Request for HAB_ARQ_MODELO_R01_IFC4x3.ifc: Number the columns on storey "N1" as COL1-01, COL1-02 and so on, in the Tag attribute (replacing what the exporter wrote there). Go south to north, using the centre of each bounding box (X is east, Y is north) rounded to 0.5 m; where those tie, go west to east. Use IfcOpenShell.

First a look at what the model holds.

```python
import ifcopenshell
import ifcopenshell.util.element
import ifcopenshell.util.placement

model = ifcopenshell.open("HAB_ARQ_MODELO_R01_IFC4x3.ifc")
print(model.schema)
storey = next(s for s in model.by_type("IfcBuildingStorey") if s.Name == "N1")
columns = [e for e in ifcopenshell.util.element.get_decomposition(storey) if e.is_a("IfcColumn")]
for e in sorted(columns, key=lambda e: e.id()):
    origin = ifcopenshell.util.placement.get_local_placement(e.ObjectPlacement)[:3, 3]
    print(e.id(), e.Tag, e.Name, origin.round(2) + 0.0, sep=" | ")
```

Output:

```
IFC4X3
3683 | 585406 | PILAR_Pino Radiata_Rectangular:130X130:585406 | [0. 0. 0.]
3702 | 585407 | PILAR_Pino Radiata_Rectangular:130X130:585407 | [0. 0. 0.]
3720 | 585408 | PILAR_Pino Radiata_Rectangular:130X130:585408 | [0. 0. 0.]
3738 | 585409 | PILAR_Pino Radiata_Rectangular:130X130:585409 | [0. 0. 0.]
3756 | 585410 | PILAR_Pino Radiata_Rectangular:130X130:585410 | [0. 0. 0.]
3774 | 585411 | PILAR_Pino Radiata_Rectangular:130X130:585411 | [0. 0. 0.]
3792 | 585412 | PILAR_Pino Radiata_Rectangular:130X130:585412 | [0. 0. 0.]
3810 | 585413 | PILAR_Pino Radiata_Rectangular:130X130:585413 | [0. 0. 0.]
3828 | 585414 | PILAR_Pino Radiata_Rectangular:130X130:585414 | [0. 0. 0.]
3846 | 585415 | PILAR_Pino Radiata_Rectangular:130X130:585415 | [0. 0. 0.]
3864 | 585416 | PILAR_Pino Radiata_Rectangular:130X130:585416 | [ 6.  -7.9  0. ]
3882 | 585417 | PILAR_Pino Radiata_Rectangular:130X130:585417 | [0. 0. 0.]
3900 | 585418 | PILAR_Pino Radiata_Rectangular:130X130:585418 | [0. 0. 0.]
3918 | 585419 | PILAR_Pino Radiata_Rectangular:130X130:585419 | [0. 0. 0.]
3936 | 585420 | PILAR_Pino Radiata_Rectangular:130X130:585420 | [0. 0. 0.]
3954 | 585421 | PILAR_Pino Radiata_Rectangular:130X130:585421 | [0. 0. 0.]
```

```python
import ifcopenshell
import ifcopenshell.geom
import ifcopenshell.util.element
import ifcopenshell.util.shape

model = ifcopenshell.open("HAB_ARQ_MODELO_R01_IFC4x3.ifc")
settings = ifcopenshell.geom.settings()
settings.set("use-world-coords", True)


def centre(element):
    shape = ifcopenshell.geom.create_shape(settings, element)
    return ifcopenshell.util.shape.get_bbox_centroid(shape.geometry)


storey = next(s for s in model.by_type("IfcBuildingStorey") if s.Name == "N1")
columns = [e for e in ifcopenshell.util.element.get_decomposition(storey) if e.is_a("IfcColumn")]

# Insertion points can sit at a corner or the storey origin, so sort by the geometry (in metres).
centres = {e: centre(e) for e in columns}
columns.sort(key=lambda e: (round(centres[e][1] / 0.5), centres[e][0]))

for i, e in enumerate(columns, start=1):
    number = f"COL1-{i:02d}"
    e.Tag = number
    print(e.id(), number)

model.write("HAB_ARQ_MODELO_R01_IFC4x3_edited.ifc")
```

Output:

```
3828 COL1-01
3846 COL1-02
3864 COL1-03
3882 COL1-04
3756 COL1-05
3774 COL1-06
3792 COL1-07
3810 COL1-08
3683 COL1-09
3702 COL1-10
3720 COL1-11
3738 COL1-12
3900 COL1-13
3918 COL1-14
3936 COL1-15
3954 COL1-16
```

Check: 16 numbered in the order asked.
